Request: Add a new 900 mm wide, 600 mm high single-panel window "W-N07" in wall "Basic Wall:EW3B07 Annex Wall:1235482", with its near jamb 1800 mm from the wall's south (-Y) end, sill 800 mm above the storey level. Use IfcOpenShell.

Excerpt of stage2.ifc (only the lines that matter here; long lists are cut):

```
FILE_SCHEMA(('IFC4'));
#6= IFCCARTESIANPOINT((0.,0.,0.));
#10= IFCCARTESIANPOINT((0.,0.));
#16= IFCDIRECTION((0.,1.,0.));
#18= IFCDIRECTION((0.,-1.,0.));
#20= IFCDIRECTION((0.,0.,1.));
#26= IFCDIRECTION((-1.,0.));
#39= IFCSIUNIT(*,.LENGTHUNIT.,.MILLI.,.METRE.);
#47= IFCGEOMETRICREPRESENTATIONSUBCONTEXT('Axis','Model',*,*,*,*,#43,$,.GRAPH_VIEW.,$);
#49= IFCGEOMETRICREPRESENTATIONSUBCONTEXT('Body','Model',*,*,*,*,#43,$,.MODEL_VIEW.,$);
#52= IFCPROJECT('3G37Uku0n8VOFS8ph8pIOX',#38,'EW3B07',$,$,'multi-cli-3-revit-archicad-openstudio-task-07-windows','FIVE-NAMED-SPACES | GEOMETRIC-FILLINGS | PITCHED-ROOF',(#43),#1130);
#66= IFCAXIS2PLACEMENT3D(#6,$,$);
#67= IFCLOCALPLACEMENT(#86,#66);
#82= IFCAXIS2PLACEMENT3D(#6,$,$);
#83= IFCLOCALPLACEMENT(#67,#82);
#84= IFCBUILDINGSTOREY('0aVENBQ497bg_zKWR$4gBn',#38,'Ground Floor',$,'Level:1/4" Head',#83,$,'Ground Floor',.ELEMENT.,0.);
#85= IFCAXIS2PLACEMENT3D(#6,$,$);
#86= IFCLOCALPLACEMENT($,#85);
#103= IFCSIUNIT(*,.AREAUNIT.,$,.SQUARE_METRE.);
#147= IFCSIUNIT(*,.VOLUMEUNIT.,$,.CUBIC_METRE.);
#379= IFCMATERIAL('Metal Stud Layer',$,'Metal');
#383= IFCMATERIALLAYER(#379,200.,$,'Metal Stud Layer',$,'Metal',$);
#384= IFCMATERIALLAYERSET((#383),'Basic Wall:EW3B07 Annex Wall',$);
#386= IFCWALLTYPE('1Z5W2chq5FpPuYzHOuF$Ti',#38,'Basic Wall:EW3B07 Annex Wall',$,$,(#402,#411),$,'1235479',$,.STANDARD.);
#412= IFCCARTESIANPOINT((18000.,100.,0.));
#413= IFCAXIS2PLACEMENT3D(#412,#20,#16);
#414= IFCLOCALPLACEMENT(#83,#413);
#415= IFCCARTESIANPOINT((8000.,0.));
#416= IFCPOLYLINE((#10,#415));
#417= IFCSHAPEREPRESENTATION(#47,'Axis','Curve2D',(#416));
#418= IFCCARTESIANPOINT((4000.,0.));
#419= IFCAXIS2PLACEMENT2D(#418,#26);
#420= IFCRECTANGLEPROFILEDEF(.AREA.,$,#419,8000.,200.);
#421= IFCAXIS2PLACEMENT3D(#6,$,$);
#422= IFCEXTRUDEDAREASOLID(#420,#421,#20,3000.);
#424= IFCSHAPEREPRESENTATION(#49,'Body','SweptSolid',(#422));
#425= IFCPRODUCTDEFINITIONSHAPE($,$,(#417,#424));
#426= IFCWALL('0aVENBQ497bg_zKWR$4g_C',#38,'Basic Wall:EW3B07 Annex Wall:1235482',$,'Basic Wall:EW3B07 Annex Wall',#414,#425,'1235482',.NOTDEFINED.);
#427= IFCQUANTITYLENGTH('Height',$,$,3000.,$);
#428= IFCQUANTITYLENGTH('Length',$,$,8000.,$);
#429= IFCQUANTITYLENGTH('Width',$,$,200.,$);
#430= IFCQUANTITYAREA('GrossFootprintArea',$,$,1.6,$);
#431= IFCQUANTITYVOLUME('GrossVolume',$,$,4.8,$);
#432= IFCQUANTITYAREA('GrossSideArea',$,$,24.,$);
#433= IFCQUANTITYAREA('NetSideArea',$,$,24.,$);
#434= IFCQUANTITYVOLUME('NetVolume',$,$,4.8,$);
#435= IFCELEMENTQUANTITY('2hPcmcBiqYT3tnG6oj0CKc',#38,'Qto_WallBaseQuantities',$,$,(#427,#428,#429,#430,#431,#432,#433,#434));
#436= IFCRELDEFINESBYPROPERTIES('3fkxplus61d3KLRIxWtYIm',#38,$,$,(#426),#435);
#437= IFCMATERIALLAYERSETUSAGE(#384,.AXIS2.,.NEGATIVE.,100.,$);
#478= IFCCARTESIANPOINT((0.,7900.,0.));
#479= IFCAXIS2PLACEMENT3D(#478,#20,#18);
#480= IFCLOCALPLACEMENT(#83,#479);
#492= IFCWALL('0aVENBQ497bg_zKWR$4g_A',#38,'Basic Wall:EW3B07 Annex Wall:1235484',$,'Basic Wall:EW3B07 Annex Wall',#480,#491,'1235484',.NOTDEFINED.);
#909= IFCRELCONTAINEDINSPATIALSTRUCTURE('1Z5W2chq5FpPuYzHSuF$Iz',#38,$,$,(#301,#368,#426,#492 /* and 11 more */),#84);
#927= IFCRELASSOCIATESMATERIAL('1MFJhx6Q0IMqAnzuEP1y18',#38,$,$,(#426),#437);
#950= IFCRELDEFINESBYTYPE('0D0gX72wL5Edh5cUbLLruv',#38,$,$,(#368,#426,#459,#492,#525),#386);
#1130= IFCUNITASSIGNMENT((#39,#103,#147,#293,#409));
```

```python
import numpy as np
import ifcopenshell
import ifcopenshell.api.feature
import ifcopenshell.api.geometry
import ifcopenshell.api.pset
import ifcopenshell.api.root
import ifcopenshell.api.spatial
import ifcopenshell.geom
import ifcopenshell.util.element
import ifcopenshell.util.placement
import ifcopenshell.util.representation
import ifcopenshell.util.shape
import ifcopenshell.util.unit

model = ifcopenshell.open("stage2.ifc")
unit_scale = ifcopenshell.util.unit.calculate_unit_scale(model)
area_scale = ifcopenshell.util.unit.calculate_unit_scale(model, "AREAUNIT")
volume_scale = ifcopenshell.util.unit.calculate_unit_scale(model, "VOLUMEUNIT")
settings = ifcopenshell.geom.settings()


def volume(element):
    """Net volume in cubic metres, openings subtracted."""
    shape = ifcopenshell.geom.create_shape(settings, element)
    return ifcopenshell.util.shape.get_volume(shape.geometry)


wall = model.by_guid("0aVENBQ497bg_zKWR$4g_C")
storey = ifcopenshell.util.element.get_container(wall, ifc_class="IfcBuildingStorey")
context = ifcopenshell.util.representation.get_context(model, "Model", "Body", "MODEL_VIEW")
before = volume(wall)

width, height, from_end, sill = 0.9, 0.6, 1.8, 0.8  # metres

# The wall runs along its own X axis, and the end named is its -X end.
wall_shape = ifcopenshell.geom.create_shape(settings, wall)
x, y, z = ifcopenshell.util.shape.get_vertices(wall_shape.geometry).T
start = x.min() + from_end
face, thickness = float(y.min()), float(y.max() - y.min())
wall_matrix = ifcopenshell.util.placement.get_local_placement(wall.ObjectPlacement)
level = ifcopenshell.util.placement.get_local_placement(storey.ObjectPlacement)[2, 3]


def in_wall(x, y):
    """Placement at x, y metres in the wall's axes, at sill height."""
    matrix = wall_matrix.copy()
    matrix[:, 3] = wall_matrix @ np.array([x / unit_scale, y / unit_scale, 0.0, 1.0])
    matrix[2, 3] = level + sill / unit_scale
    return matrix


# Opening: a box that overshoots both wall faces by 50 mm.
opening = ifcopenshell.api.root.create_entity(model, ifc_class="IfcOpeningElement", predefined_type="OPENING")
box = ifcopenshell.api.geometry.add_wall_representation(
    model, context=context, length=width, height=height, thickness=thickness + 0.1
)
ifcopenshell.api.geometry.assign_representation(model, product=opening, representation=box)
ifcopenshell.api.geometry.edit_object_placement(model, product=opening, matrix=in_wall(start, face - 0.05), is_si=False)
ifcopenshell.api.feature.add_feature(model, feature=opening, element=wall)

window = ifcopenshell.api.root.create_entity(model, ifc_class="IfcWindow", name="W-N07", predefined_type="WINDOW")
window.OverallWidth, window.OverallHeight = width / unit_scale, height / unit_scale
window.PartitioningType = "SINGLE_PANEL"
body = ifcopenshell.api.geometry.add_window_representation(
    model,
    context=context,
    overall_width=window.OverallWidth,
    overall_height=window.OverallHeight,
    partition_type="SINGLE_PANEL",
)
ifcopenshell.api.geometry.assign_representation(model, product=window, representation=body)
ifcopenshell.api.spatial.assign_container(model, products=[window], relating_structure=storey)
ifcopenshell.api.feature.add_filling(model, opening=opening, element=window)

# Centre the window in the wall's thickness.
ifcopenshell.api.geometry.edit_object_placement(model, product=window, matrix=in_wall(start, face), is_si=False)
window_shape = ifcopenshell.geom.create_shape(settings, window)
depth = ifcopenshell.util.shape.get_vertices(window_shape.geometry)[:, 1]
offset = face + thickness / 2 - (depth.min() + depth.max()) / 2
ifcopenshell.api.geometry.edit_object_placement(model, product=window, matrix=in_wall(start, offset), is_si=False)

after = volume(wall)

# Update the wall's stored quantities.
qto = model.by_id(ifcopenshell.util.element.get_pset(wall, "Qto_WallBaseQuantities", should_inherit=False)["id"])
ifcopenshell.api.pset.edit_qto(model, qto=qto, properties={
    "NetSideArea": after / thickness / area_scale,
    "NetVolume": after / volume_scale,
})

print(f"wall volume {before:.3f} -> {after:.3f} m3")

model.write("stage2_rev.ifc")
```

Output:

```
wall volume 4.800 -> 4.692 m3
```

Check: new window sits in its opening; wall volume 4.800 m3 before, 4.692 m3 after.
